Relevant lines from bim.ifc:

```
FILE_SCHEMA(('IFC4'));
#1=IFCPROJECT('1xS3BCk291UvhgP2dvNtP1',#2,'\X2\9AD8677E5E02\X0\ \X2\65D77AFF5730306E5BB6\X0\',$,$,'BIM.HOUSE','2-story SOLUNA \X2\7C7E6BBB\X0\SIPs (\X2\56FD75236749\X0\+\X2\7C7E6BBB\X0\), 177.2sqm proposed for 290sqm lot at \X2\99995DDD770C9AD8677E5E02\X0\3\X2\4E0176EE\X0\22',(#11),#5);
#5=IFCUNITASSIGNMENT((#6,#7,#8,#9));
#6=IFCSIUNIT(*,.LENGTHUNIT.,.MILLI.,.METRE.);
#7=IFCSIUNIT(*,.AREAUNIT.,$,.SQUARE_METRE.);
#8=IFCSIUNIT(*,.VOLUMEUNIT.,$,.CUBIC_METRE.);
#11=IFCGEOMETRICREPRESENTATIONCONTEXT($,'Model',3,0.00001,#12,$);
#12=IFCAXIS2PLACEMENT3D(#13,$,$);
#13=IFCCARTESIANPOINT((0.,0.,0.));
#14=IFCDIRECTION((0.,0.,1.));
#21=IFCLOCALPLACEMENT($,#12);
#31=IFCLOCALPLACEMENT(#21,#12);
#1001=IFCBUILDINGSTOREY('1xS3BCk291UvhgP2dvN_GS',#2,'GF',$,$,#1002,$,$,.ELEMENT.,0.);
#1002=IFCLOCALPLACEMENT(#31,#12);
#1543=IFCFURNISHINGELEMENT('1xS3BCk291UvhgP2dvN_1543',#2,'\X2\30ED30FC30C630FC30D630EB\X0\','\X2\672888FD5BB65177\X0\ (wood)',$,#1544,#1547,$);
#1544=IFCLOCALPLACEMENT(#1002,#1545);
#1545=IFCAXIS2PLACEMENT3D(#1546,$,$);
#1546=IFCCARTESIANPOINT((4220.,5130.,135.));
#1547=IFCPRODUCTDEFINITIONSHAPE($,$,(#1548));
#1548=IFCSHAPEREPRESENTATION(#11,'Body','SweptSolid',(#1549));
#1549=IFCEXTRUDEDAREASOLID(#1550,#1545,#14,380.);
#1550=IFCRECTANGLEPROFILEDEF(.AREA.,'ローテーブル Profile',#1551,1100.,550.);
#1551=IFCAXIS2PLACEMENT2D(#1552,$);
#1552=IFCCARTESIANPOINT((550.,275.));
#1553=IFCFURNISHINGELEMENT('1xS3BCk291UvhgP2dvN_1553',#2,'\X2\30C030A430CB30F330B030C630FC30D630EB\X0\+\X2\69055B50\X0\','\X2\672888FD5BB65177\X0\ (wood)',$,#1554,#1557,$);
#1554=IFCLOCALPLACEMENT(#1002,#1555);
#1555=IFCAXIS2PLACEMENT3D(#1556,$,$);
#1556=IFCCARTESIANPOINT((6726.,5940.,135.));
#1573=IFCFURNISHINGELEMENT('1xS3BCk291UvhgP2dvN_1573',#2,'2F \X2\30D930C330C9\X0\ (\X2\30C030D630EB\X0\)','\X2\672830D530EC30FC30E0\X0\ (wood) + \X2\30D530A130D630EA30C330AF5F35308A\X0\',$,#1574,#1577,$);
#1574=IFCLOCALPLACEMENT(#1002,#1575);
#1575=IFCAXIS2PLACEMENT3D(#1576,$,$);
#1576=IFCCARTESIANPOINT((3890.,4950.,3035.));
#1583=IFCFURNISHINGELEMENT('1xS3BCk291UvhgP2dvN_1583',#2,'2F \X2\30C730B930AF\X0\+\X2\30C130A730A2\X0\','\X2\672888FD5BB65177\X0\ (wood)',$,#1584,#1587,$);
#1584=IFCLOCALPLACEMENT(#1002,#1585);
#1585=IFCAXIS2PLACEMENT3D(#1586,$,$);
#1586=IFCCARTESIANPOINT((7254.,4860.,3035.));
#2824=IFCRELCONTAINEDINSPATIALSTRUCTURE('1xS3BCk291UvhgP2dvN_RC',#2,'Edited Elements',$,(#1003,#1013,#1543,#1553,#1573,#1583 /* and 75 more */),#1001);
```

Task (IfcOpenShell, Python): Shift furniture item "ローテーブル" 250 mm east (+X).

```python
import ifcopenshell
import ifcopenshell.api.geometry
import ifcopenshell.util.placement
import ifcopenshell.util.unit

model = ifcopenshell.open("bim.ifc")
unit_scale = ifcopenshell.util.unit.calculate_unit_scale(model)

item = model.by_guid("1xS3BCk291UvhgP2dvN_1543")
matrix = ifcopenshell.util.placement.get_local_placement(item.ObjectPlacement)
matrix[0, 3] += 0.25 / unit_scale
ifcopenshell.api.geometry.edit_object_placement(model, product=item, matrix=matrix, is_si=False)

print(ifcopenshell.util.placement.get_local_placement(item.ObjectPlacement).round(3) + 0.0)

model.write("bim_edited.ifc")
```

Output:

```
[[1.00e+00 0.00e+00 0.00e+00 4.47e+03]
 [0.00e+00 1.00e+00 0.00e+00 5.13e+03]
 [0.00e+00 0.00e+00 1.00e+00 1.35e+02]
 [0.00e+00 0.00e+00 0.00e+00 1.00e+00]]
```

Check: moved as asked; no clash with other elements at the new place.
